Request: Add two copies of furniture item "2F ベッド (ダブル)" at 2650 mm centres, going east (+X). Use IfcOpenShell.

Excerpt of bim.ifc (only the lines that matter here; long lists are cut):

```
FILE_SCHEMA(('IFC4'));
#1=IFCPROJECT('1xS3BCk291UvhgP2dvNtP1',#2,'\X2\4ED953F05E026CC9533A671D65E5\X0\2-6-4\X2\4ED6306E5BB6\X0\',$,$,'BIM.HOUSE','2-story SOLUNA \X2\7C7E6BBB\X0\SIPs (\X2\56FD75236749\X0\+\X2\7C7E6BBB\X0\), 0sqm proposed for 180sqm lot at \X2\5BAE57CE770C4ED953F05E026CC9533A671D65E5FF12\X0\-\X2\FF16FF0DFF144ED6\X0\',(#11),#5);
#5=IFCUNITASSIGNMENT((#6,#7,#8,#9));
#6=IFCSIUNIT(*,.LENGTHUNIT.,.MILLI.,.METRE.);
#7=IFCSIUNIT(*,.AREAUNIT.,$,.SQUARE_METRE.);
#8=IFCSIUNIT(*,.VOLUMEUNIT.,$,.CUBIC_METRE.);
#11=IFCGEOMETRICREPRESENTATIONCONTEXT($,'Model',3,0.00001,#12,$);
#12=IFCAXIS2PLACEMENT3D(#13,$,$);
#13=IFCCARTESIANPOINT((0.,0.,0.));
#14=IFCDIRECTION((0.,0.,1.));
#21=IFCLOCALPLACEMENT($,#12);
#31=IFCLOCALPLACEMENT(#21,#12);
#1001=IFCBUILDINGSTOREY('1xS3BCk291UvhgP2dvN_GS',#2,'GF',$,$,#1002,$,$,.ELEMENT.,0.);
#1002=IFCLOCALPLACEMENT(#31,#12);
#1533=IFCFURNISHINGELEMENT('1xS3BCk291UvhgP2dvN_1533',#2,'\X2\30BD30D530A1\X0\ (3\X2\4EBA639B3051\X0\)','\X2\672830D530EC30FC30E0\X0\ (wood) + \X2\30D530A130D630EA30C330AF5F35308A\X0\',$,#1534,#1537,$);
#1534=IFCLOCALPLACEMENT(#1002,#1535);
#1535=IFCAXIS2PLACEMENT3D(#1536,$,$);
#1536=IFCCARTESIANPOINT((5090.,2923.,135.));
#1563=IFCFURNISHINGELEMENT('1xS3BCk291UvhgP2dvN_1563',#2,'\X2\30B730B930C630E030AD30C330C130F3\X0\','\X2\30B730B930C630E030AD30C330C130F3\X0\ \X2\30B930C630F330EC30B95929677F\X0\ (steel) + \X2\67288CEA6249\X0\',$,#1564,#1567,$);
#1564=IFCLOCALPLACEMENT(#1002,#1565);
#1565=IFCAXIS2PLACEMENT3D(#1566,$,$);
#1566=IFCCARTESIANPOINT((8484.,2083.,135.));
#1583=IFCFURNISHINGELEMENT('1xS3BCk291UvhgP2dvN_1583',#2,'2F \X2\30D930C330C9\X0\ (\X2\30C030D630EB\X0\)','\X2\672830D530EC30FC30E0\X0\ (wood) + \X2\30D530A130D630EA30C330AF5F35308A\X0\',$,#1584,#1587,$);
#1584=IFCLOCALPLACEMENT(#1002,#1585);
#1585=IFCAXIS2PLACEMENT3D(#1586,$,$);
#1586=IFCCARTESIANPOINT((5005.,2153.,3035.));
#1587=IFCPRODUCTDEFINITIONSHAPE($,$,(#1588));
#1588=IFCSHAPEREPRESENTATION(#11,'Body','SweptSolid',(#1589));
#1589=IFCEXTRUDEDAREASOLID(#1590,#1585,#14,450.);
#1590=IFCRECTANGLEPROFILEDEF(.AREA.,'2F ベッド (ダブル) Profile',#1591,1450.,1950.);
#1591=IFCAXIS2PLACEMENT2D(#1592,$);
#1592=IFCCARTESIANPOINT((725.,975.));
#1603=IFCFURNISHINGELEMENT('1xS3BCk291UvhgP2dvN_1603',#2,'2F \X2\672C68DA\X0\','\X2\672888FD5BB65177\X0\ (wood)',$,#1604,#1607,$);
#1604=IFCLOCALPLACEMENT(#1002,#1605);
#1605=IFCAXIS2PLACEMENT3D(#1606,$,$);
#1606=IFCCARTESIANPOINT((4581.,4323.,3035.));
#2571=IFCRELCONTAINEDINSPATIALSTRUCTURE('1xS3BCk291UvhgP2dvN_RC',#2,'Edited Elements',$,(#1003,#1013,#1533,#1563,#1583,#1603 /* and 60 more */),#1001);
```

```python
import numpy as np
import ifcopenshell
import ifcopenshell.api.geometry
import ifcopenshell.api.root
import ifcopenshell.util.element
import ifcopenshell.util.placement
import ifcopenshell.util.unit

model = ifcopenshell.open("bim.ifc")
unit_scale = ifcopenshell.util.unit.calculate_unit_scale(model)


def reuse_history(source, copy):
    """copy_class also copies each property set's owner history, people and application; keep the originals."""
    for rel in copy.IsDefinedBy:
        if rel.is_a("IfcRelDefinesByProperties") and (history := rel.RelatingPropertyDefinition.OwnerHistory):
            rel.RelatingPropertyDefinition.OwnerHistory = source.OwnerHistory
            ifcopenshell.util.element.remove_deep2(model, history)


source = model.by_guid("1xS3BCk291UvhgP2dvN_1583")
base = ifcopenshell.util.placement.get_local_placement(source.ObjectPlacement)
step = np.array([1.0, 0.0, 0.0]) * 2.65 / unit_scale

for i in range(1, 3):
    copy = ifcopenshell.api.root.copy_class(model, product=source)
    copy.Representation = ifcopenshell.util.element.copy_deep(
        model, source.Representation, exclude=["IfcGeometricRepresentationContext", "IfcRepresentationMap"]
    )
    reuse_history(source, copy)
    matrix = base.copy()
    matrix[:3, 3] += i * step
    print("added at", matrix[:3, 3].round(3) + 0.0)
    ifcopenshell.api.geometry.edit_object_placement(model, product=copy, matrix=matrix, is_si=False)

model.write("bim_rev.ifc")
```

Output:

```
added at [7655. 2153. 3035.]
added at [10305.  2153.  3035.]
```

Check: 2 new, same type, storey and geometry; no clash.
